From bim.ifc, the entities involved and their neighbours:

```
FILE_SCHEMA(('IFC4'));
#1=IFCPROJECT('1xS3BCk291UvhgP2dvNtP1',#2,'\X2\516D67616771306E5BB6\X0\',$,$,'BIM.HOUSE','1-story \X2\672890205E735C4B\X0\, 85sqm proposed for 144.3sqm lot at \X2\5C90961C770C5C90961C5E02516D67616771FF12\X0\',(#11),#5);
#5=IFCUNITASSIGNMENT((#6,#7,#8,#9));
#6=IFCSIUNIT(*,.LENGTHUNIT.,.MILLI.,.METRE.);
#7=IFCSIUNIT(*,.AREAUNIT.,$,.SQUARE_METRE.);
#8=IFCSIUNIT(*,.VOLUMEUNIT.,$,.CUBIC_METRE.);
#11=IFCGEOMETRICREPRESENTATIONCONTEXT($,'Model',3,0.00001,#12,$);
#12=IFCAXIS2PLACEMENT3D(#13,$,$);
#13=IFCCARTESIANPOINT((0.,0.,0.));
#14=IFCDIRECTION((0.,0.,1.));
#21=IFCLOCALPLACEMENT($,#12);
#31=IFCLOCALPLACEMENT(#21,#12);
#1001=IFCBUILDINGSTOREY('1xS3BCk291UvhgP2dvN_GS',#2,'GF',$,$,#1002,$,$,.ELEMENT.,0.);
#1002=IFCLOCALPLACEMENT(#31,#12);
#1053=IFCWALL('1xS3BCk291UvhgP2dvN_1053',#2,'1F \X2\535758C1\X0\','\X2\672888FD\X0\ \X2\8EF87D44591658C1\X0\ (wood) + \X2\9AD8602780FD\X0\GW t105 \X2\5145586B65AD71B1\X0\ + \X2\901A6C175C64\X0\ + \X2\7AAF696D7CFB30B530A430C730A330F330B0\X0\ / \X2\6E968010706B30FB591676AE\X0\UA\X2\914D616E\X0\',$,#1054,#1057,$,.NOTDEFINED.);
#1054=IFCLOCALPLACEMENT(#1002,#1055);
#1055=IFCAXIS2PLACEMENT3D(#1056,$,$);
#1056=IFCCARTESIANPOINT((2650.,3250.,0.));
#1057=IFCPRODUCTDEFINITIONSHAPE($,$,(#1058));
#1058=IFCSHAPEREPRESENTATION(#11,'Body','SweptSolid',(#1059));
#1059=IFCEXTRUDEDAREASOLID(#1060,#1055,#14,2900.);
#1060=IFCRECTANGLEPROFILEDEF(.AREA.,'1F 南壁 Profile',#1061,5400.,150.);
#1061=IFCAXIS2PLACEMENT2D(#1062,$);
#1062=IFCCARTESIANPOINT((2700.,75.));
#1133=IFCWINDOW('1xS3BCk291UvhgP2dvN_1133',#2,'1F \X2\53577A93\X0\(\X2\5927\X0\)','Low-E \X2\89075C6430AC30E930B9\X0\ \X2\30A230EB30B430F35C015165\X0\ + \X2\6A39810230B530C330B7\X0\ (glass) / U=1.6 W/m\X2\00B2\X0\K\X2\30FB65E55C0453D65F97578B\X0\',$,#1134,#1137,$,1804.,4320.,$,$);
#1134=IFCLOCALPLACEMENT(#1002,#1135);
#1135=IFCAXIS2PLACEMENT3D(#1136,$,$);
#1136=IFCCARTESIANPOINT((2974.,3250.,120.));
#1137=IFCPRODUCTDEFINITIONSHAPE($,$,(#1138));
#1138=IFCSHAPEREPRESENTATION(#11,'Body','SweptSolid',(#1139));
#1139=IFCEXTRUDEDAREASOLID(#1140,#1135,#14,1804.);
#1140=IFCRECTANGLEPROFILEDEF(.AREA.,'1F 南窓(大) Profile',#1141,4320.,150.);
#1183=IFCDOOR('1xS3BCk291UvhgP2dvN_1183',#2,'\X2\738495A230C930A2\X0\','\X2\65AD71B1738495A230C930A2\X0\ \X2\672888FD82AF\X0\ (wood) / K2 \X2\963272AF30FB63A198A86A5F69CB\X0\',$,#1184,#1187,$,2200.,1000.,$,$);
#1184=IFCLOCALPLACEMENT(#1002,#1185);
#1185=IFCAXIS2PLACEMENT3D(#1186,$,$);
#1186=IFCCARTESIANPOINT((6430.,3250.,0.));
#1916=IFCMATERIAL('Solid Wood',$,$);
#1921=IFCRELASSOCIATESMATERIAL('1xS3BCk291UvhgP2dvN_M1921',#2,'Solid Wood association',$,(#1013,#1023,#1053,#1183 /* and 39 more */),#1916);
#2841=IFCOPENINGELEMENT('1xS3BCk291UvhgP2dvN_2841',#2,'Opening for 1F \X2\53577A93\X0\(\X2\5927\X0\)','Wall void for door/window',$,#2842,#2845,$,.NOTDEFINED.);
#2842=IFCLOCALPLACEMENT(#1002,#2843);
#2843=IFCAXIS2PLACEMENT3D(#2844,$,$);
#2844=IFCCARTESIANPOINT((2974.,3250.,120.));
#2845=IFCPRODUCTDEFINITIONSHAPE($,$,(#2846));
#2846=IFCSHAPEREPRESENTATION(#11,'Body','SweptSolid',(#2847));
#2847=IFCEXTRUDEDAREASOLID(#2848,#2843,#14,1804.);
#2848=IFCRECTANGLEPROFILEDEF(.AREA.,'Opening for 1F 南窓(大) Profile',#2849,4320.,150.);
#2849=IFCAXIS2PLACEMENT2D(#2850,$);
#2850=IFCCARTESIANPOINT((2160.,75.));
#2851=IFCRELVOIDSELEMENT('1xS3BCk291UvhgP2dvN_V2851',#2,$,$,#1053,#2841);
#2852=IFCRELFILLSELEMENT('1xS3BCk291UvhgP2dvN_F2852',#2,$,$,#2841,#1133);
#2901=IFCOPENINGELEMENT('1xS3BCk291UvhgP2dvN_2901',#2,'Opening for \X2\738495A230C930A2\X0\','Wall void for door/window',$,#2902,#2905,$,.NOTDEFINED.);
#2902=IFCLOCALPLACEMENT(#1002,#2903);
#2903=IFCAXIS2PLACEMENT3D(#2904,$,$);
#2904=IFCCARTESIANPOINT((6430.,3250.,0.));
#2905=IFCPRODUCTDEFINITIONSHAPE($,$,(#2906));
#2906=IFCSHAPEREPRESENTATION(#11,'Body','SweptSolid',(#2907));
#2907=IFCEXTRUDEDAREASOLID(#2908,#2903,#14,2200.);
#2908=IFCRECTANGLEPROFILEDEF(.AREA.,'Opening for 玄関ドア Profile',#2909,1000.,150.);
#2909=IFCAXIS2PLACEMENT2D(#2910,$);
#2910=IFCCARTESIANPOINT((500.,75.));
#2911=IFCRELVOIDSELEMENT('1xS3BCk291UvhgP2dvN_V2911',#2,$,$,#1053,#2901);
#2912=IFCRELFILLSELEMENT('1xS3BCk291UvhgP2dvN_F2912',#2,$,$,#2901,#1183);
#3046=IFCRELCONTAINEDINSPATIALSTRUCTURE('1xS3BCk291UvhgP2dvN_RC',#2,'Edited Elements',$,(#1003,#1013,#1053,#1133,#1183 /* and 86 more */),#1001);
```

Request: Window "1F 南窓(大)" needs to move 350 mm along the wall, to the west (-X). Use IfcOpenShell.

```python
import ifcopenshell
import ifcopenshell.api.geometry
import ifcopenshell.util.placement
import ifcopenshell.util.unit

model = ifcopenshell.open("bim.ifc")
unit_scale = ifcopenshell.util.unit.calculate_unit_scale(model)

window = model.by_guid("1xS3BCk291UvhgP2dvN_1133")
opening = window.FillsVoids[0].RelatingOpeningElement
wall = opening.VoidsElements[0].RelatingBuildingElement

wall_matrix = ifcopenshell.util.placement.get_local_placement(wall.ObjectPlacement)
shift = wall_matrix[:3, 0] * -0.35 / unit_scale
before = ifcopenshell.util.placement.get_local_placement(window.ObjectPlacement)[:3, 3].copy()

# The window is not placed relative to its opening, so move both.
for product in (opening, window):
    matrix = ifcopenshell.util.placement.get_local_placement(product.ObjectPlacement)
    matrix[:3, 3] += shift
    ifcopenshell.api.geometry.edit_object_placement(model, product=product, matrix=matrix, is_si=False)

after = ifcopenshell.util.placement.get_local_placement(window.ObjectPlacement)[:3, 3]
print("window moved by", (after - before).round(3) + 0.0)

model.write("bim_updated.ifc")
```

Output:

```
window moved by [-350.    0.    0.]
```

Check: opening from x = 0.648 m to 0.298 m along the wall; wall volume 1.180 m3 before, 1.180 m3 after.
